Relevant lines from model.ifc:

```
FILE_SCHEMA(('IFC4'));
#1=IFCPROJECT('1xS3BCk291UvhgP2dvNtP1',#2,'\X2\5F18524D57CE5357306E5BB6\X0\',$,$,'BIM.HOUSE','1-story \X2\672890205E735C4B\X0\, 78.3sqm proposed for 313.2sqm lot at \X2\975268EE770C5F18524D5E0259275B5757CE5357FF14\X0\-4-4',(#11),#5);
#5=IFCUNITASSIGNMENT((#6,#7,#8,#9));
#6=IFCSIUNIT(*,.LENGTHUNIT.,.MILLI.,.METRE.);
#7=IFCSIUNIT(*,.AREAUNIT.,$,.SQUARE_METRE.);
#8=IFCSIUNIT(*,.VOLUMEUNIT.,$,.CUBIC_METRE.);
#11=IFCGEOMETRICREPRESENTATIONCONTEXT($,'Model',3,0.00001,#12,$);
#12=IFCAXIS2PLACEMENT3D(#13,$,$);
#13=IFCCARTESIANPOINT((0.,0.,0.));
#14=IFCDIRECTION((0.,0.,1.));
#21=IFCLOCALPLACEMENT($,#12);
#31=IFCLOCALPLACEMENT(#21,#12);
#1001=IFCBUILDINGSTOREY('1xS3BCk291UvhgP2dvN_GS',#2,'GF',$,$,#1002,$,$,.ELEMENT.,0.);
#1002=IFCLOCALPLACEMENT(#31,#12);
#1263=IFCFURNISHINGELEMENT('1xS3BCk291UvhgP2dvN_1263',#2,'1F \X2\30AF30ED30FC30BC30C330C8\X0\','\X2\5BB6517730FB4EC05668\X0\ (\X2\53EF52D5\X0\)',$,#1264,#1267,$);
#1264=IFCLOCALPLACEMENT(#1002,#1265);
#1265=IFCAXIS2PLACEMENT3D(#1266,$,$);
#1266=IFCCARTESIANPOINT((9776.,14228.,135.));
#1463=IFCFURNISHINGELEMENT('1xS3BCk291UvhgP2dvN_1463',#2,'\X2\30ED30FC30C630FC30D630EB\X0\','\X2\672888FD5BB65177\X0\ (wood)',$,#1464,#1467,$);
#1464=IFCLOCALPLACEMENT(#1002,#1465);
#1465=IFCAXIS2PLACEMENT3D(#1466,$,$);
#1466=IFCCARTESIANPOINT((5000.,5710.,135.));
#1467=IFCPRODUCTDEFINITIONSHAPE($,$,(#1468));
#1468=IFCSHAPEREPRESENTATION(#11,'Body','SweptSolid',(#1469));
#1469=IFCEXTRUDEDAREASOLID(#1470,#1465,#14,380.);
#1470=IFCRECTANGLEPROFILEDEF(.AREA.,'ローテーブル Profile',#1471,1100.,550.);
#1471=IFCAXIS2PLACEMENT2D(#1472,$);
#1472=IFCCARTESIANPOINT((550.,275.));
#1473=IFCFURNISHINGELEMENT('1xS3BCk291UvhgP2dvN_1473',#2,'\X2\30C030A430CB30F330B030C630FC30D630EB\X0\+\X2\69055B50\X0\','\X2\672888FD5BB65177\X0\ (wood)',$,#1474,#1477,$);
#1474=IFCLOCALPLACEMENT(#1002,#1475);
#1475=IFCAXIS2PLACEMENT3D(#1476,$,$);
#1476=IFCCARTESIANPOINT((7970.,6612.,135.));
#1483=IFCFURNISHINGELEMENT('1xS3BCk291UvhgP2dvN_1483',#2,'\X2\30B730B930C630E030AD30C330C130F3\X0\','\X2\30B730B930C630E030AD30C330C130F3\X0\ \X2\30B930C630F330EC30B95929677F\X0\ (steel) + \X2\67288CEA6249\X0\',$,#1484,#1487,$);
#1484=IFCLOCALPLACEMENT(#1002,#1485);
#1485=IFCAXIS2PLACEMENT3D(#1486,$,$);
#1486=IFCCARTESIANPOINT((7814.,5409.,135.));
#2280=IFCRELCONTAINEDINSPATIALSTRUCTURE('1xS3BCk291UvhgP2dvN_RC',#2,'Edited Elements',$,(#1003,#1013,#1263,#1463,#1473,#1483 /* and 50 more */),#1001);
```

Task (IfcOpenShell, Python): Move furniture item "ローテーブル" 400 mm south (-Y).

```python
import ifcopenshell
import ifcopenshell.api.geometry
import ifcopenshell.util.placement

model = ifcopenshell.open("model.ifc")

item = model.by_id(1463)
matrix = ifcopenshell.util.placement.get_local_placement(item.ObjectPlacement)
matrix[1, 3] -= 400.0
ifcopenshell.api.geometry.edit_object_placement(model, product=item, matrix=matrix, is_si=False)

print(ifcopenshell.util.placement.get_local_placement(item.ObjectPlacement).round(3) + 0.0)

model.write("model_updated.ifc")
```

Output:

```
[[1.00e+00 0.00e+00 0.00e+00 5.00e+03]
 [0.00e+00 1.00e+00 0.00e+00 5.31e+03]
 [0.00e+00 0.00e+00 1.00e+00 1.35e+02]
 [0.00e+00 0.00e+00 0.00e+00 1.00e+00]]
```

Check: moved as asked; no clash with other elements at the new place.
